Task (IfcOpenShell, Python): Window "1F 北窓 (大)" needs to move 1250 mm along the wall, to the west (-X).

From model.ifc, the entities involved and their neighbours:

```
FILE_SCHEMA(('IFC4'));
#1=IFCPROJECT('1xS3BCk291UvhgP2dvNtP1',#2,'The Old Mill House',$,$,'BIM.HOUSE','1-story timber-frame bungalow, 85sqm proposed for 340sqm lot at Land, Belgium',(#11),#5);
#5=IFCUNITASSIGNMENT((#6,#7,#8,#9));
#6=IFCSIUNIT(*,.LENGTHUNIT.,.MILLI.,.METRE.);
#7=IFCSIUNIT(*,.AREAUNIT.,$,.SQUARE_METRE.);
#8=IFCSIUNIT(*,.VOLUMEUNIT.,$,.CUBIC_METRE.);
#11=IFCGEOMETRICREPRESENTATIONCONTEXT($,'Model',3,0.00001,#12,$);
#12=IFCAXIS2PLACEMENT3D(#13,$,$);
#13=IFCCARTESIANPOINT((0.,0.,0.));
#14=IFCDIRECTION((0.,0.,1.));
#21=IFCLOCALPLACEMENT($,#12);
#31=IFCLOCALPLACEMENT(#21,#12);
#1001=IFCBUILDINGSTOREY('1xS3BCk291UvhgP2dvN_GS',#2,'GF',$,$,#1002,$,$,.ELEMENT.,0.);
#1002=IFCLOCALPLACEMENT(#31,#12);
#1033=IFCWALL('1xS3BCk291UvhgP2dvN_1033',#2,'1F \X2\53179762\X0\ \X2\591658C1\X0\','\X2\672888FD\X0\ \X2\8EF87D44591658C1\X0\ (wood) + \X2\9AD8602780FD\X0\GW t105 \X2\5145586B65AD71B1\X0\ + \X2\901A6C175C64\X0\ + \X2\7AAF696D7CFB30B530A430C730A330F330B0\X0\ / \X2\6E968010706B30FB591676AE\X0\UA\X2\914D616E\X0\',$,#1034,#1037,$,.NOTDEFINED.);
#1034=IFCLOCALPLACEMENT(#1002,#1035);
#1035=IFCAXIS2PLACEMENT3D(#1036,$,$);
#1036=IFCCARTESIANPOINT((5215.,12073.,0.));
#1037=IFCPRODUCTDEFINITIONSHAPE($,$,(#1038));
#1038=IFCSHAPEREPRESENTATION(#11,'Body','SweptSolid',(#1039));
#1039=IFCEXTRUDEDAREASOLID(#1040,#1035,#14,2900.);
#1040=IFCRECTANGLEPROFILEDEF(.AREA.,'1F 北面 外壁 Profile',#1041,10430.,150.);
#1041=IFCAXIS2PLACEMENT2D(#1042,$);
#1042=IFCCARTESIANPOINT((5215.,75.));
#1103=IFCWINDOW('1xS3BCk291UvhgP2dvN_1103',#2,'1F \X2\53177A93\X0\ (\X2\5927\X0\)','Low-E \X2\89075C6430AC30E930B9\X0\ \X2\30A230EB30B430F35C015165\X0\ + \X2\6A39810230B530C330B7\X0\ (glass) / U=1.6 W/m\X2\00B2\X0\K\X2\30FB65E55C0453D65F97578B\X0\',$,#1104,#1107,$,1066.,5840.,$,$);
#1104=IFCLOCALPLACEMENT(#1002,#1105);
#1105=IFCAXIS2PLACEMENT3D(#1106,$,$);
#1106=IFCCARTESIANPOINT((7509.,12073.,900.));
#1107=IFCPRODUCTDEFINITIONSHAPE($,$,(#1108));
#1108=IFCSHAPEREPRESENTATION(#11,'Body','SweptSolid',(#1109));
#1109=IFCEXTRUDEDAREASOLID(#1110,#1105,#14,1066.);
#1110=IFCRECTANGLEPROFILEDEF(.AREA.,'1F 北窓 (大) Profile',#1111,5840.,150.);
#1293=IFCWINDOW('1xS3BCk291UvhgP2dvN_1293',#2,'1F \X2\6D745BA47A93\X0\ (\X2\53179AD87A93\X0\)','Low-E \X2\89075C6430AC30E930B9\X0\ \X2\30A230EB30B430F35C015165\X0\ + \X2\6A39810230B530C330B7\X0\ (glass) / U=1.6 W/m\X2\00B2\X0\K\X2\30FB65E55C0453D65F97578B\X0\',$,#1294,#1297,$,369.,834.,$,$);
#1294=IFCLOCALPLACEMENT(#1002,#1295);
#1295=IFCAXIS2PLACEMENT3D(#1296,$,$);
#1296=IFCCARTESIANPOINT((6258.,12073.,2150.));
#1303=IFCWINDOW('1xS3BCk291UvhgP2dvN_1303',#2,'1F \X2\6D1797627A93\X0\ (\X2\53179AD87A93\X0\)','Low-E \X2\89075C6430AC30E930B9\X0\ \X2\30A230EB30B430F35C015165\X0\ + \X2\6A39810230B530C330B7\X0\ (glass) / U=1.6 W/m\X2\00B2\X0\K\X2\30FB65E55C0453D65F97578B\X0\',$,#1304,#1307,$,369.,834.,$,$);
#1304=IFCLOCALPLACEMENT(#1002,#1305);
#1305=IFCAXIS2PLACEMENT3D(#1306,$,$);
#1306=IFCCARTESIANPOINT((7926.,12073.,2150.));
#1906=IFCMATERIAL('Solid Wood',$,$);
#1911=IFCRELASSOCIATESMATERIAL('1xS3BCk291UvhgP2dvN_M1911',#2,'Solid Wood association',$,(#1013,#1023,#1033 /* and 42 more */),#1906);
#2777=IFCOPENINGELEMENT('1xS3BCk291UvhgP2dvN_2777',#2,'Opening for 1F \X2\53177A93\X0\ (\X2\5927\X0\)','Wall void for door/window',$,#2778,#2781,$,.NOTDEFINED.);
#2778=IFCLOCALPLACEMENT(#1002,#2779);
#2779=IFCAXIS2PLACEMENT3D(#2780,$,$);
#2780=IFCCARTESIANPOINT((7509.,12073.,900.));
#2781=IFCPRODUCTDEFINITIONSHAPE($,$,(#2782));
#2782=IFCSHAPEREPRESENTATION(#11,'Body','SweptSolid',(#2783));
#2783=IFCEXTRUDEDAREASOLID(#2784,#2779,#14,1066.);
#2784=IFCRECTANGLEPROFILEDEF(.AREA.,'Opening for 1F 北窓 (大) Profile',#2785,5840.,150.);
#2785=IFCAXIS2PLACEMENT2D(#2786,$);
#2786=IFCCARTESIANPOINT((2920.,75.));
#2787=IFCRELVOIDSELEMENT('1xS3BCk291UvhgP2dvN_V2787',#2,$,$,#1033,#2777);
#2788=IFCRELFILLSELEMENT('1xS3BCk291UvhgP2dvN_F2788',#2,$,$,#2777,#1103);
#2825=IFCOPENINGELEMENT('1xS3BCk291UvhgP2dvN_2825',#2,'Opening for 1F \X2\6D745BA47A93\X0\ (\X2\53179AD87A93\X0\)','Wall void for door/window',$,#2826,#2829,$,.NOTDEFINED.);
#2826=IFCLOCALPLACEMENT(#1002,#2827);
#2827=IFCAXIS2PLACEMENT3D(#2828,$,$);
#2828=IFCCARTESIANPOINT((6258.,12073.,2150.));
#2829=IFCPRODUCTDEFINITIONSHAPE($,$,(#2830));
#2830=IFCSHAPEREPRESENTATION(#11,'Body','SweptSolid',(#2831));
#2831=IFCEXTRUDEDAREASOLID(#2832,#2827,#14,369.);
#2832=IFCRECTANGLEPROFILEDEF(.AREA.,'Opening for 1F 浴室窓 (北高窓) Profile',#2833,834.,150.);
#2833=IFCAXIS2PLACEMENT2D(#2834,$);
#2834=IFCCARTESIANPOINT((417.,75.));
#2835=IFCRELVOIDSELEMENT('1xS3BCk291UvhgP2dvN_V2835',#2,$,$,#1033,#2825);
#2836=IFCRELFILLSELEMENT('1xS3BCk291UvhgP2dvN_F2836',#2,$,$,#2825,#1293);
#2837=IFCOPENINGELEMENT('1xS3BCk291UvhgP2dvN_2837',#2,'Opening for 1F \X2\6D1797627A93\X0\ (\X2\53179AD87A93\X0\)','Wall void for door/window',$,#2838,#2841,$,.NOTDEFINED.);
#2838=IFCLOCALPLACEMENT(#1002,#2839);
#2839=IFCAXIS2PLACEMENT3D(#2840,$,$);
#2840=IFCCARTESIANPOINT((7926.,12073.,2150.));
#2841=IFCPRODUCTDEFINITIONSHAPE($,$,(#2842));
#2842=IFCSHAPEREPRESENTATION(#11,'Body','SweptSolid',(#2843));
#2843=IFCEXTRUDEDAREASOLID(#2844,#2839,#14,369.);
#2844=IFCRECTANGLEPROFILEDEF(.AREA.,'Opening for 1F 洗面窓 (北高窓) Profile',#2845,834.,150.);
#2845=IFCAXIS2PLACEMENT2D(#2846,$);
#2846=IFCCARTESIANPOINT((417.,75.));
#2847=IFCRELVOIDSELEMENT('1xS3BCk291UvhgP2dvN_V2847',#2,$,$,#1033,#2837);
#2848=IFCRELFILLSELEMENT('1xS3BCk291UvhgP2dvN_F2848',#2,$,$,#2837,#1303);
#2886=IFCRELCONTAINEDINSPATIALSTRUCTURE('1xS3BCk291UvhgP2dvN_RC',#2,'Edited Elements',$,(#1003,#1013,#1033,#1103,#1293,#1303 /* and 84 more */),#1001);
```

```python
import ifcopenshell
import ifcopenshell.api.geometry
import ifcopenshell.util.placement
import ifcopenshell.util.unit

model = ifcopenshell.open("model.ifc")
unit_scale = ifcopenshell.util.unit.calculate_unit_scale(model)

window = model.by_guid("1xS3BCk291UvhgP2dvN_1103")
opening = window.FillsVoids[0].RelatingOpeningElement
wall = opening.VoidsElements[0].RelatingBuildingElement

wall_matrix = ifcopenshell.util.placement.get_local_placement(wall.ObjectPlacement)
shift = wall_matrix[:3, 0] * -1.25 / unit_scale
before = ifcopenshell.util.placement.get_local_placement(window.ObjectPlacement)[:3, 3].copy()

# The window is not placed relative to its opening, so move both.
for product in (opening, window):
    matrix = ifcopenshell.util.placement.get_local_placement(product.ObjectPlacement)
    matrix[:3, 3] += shift
    ifcopenshell.api.geometry.edit_object_placement(model, product=product, matrix=matrix, is_si=False)

after = ifcopenshell.util.placement.get_local_placement(window.ObjectPlacement)[:3, 3]
print("window moved by", (after - before).round(3) + 0.0)

model.write("model-out.ifc")
```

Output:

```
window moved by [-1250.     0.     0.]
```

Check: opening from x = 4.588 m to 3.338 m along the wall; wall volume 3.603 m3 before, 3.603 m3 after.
